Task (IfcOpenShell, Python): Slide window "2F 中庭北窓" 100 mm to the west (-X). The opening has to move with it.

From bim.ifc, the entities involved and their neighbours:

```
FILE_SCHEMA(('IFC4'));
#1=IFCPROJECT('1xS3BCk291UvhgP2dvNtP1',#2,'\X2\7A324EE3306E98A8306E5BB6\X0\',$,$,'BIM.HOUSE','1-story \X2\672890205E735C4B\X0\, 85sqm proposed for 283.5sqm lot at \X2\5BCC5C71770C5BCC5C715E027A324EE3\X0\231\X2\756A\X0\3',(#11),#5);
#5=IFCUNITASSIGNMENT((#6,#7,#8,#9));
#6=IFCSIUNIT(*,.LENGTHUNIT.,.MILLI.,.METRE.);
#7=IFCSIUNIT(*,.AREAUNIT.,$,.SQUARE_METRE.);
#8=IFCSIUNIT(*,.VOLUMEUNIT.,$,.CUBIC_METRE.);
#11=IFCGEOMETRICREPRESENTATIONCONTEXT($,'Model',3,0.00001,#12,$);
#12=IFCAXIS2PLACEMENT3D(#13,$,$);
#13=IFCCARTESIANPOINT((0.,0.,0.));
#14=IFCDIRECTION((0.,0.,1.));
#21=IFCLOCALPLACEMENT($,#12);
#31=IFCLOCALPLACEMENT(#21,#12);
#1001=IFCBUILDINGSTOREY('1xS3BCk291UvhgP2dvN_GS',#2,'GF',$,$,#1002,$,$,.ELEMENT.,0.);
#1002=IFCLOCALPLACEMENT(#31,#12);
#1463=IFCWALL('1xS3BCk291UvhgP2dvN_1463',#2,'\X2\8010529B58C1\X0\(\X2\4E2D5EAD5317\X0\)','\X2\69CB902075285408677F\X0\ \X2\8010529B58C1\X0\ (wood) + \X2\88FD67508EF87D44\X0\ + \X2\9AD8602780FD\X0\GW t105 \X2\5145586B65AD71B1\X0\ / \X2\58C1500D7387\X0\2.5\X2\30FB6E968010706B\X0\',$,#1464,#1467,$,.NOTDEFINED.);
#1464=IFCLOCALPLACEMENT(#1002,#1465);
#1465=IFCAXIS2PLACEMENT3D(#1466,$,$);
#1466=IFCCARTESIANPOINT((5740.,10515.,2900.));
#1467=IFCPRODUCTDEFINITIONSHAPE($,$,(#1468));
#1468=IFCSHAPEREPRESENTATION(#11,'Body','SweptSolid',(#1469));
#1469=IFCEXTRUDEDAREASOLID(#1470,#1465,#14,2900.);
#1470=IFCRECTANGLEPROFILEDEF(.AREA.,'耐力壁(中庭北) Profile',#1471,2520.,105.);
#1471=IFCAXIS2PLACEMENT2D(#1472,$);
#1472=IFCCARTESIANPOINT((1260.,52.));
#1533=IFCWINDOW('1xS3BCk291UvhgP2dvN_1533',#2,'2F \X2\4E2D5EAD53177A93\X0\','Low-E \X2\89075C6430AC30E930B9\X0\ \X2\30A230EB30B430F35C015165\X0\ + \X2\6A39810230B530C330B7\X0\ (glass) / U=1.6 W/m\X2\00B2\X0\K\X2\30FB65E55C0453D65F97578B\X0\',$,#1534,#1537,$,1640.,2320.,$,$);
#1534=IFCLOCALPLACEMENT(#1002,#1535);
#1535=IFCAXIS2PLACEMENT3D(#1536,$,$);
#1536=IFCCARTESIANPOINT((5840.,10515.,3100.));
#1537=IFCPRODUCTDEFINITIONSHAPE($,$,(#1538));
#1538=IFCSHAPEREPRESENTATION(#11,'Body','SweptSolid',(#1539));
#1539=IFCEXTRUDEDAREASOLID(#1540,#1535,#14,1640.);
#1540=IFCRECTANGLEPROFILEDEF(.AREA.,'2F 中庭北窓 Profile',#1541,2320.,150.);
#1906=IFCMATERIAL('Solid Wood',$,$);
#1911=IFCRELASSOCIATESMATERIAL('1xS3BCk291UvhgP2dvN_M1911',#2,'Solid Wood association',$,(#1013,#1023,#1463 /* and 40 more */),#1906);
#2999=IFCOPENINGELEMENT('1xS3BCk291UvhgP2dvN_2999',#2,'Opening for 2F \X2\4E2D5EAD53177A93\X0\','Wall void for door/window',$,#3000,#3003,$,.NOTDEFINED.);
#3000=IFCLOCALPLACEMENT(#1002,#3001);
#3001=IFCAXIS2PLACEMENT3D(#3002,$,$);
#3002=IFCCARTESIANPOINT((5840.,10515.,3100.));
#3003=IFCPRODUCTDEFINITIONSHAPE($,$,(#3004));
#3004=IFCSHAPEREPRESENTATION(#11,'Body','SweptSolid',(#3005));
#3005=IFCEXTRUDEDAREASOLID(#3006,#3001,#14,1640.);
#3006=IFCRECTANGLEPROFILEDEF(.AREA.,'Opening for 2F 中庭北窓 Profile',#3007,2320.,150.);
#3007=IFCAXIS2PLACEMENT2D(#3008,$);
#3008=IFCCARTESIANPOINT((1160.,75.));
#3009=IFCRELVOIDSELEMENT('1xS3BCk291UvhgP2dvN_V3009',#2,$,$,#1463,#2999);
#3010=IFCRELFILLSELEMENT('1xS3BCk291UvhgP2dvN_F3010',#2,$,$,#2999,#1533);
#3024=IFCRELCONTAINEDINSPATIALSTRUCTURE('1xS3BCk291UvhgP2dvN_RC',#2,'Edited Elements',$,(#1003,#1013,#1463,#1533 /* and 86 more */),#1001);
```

```python
import ifcopenshell
import ifcopenshell.api.geometry
import ifcopenshell.util.placement
import ifcopenshell.util.unit

model = ifcopenshell.open("bim.ifc")
unit_scale = ifcopenshell.util.unit.calculate_unit_scale(model)

window = model.by_id(1533)
opening = window.FillsVoids[0].RelatingOpeningElement
wall = opening.VoidsElements[0].RelatingBuildingElement

wall_matrix = ifcopenshell.util.placement.get_local_placement(wall.ObjectPlacement)
shift = wall_matrix[:3, 0] * -0.1 / unit_scale
before = ifcopenshell.util.placement.get_local_placement(window.ObjectPlacement)[:3, 3].copy()

# The window is not placed relative to its opening, so move both.
for product in (opening, window):
    matrix = ifcopenshell.util.placement.get_local_placement(product.ObjectPlacement)
    matrix[:3, 3] += shift
    ifcopenshell.api.geometry.edit_object_placement(model, product=product, matrix=matrix, is_si=False)

after = ifcopenshell.util.placement.get_local_placement(window.ObjectPlacement)[:3, 3]
print("window moved by", (after - before).round(3) + 0.0)

model.write("bim-out.ifc")
```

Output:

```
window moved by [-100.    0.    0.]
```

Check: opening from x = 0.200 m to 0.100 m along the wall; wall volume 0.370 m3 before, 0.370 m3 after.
